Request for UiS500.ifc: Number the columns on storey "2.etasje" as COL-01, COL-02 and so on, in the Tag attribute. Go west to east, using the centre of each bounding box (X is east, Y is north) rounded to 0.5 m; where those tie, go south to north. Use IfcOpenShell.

First a look at what the model holds.

```python
import ifcopenshell
import ifcopenshell.util.element
import ifcopenshell.util.placement

model = ifcopenshell.open("UiS500.ifc")
print(model.schema)
storey = next(s for s in model.by_type("IfcBuildingStorey") if s.Name == "2.etasje")
columns = [e for e in ifcopenshell.util.element.get_decomposition(storey) if e.is_a("IfcColumn")]
for e in sorted(columns, key=lambda e: e.id()):
    origin = ifcopenshell.util.placement.get_local_placement(e.ObjectPlacement)[:3, 3]
    print(e.id(), e.Tag, e.Name, origin.round(2) + 0.0, sep=" | ")
```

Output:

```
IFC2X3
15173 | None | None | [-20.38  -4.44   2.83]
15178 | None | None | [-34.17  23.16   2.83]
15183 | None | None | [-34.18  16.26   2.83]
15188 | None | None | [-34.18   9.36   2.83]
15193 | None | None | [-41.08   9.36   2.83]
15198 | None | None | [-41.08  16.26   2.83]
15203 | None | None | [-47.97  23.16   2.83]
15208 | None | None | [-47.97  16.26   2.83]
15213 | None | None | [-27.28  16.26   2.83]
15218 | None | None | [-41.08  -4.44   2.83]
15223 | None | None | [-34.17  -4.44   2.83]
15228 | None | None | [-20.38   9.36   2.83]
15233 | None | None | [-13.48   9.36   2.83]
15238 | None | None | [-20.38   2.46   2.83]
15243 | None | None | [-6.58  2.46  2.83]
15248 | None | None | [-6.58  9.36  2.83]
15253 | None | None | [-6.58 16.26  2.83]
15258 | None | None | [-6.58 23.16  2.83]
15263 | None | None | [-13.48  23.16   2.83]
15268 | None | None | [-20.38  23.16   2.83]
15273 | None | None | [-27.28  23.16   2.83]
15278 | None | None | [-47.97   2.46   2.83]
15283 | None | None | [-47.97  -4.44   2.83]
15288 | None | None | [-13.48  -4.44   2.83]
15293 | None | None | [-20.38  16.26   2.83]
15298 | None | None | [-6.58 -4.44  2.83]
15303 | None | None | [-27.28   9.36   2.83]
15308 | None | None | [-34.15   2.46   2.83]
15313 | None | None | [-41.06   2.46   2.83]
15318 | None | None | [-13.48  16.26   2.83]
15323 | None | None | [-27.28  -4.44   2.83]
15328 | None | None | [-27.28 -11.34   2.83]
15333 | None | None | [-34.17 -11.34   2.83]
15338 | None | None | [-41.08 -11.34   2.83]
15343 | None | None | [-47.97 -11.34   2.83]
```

```python
import ifcopenshell
import ifcopenshell.geom
import ifcopenshell.util.element
import ifcopenshell.util.shape

model = ifcopenshell.open("UiS500.ifc")
settings = ifcopenshell.geom.settings()
settings.set("use-world-coords", True)


def centre(element):
    shape = ifcopenshell.geom.create_shape(settings, element)
    return ifcopenshell.util.shape.get_bbox_centroid(shape.geometry)


storey = next(s for s in model.by_type("IfcBuildingStorey") if s.Name == "2.etasje")
columns = [e for e in ifcopenshell.util.element.get_decomposition(storey) if e.is_a("IfcColumn")]

# Insertion points can sit at a corner or the storey origin, so sort by the geometry (in metres).
centres = {e: centre(e) for e in columns}
columns.sort(key=lambda e: (round(centres[e][0] / 0.5), centres[e][1]))

for i, e in enumerate(columns, start=1):
    number = f"COL-{i:02d}"
    e.Tag = number
    print(e.id(), number)

model.write("UiS500-out.ifc")
```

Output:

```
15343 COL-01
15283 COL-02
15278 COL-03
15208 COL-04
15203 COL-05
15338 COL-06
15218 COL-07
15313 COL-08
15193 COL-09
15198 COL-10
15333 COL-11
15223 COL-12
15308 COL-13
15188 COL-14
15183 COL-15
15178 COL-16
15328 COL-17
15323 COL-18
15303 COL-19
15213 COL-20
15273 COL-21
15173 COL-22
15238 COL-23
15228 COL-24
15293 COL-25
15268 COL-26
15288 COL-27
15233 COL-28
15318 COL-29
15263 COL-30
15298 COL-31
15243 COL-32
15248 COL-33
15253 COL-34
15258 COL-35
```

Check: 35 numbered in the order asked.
